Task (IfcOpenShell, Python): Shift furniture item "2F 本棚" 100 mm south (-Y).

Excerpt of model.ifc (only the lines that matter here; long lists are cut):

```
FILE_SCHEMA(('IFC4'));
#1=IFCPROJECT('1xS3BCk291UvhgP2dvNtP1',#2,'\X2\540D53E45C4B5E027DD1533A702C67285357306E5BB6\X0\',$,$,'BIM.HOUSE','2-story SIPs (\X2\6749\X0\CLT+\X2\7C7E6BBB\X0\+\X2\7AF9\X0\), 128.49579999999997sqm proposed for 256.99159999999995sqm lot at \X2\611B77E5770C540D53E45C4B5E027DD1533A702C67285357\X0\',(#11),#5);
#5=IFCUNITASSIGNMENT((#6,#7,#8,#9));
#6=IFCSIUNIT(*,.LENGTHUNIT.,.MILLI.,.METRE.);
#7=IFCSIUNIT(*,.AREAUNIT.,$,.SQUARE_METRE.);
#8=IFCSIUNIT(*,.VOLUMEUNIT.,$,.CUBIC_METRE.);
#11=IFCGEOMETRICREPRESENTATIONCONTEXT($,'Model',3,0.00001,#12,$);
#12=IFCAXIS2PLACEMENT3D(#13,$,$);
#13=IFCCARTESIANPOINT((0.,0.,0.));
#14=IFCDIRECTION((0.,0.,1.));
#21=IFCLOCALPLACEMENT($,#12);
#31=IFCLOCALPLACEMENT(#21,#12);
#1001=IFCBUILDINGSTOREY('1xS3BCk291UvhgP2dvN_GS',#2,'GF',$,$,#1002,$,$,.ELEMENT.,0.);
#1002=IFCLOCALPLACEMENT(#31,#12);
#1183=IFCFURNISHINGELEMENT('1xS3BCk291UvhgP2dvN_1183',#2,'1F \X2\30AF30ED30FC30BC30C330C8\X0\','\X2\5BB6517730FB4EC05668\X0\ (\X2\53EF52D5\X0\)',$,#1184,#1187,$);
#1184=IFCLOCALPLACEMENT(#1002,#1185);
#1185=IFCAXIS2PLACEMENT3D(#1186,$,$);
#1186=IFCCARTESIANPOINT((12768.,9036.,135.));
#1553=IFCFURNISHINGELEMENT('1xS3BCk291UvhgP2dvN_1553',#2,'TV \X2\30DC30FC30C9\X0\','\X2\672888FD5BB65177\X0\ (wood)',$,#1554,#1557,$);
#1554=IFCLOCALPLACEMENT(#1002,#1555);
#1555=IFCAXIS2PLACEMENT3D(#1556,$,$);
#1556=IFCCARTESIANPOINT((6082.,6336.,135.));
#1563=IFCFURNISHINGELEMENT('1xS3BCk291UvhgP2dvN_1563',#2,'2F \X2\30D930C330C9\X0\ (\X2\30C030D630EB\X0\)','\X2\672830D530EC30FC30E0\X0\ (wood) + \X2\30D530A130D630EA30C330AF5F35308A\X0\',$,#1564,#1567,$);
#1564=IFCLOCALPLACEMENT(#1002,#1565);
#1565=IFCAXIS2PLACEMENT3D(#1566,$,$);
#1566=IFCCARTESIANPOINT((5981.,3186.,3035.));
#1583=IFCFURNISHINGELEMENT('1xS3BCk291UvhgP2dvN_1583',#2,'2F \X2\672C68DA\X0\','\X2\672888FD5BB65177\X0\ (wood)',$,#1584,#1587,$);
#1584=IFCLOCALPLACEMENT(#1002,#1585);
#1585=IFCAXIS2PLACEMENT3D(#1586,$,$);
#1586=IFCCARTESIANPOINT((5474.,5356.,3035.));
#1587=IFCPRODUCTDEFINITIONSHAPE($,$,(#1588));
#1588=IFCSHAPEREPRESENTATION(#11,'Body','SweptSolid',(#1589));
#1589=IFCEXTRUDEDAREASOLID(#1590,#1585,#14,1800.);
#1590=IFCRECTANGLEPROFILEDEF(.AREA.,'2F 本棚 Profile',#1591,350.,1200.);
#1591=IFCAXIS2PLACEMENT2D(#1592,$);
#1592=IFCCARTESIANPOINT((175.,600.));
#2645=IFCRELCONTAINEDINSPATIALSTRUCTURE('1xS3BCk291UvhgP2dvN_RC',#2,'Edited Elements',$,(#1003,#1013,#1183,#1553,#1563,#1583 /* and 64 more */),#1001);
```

```python
import ifcopenshell
import ifcopenshell.api.geometry
import ifcopenshell.util.placement
import ifcopenshell.util.unit

model = ifcopenshell.open("model.ifc")
unit_scale = ifcopenshell.util.unit.calculate_unit_scale(model)

item = model.by_guid("1xS3BCk291UvhgP2dvN_1583")
matrix = ifcopenshell.util.placement.get_local_placement(item.ObjectPlacement)
matrix[1, 3] -= 0.1 / unit_scale
ifcopenshell.api.geometry.edit_object_placement(model, product=item, matrix=matrix, is_si=False)

print(ifcopenshell.util.placement.get_local_placement(item.ObjectPlacement).round(3) + 0.0)

model.write("model-out.ifc")
```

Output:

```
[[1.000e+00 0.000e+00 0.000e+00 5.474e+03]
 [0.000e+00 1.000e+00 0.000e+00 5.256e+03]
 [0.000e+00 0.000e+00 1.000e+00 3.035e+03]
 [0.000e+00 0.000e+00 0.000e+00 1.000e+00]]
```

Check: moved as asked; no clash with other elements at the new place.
